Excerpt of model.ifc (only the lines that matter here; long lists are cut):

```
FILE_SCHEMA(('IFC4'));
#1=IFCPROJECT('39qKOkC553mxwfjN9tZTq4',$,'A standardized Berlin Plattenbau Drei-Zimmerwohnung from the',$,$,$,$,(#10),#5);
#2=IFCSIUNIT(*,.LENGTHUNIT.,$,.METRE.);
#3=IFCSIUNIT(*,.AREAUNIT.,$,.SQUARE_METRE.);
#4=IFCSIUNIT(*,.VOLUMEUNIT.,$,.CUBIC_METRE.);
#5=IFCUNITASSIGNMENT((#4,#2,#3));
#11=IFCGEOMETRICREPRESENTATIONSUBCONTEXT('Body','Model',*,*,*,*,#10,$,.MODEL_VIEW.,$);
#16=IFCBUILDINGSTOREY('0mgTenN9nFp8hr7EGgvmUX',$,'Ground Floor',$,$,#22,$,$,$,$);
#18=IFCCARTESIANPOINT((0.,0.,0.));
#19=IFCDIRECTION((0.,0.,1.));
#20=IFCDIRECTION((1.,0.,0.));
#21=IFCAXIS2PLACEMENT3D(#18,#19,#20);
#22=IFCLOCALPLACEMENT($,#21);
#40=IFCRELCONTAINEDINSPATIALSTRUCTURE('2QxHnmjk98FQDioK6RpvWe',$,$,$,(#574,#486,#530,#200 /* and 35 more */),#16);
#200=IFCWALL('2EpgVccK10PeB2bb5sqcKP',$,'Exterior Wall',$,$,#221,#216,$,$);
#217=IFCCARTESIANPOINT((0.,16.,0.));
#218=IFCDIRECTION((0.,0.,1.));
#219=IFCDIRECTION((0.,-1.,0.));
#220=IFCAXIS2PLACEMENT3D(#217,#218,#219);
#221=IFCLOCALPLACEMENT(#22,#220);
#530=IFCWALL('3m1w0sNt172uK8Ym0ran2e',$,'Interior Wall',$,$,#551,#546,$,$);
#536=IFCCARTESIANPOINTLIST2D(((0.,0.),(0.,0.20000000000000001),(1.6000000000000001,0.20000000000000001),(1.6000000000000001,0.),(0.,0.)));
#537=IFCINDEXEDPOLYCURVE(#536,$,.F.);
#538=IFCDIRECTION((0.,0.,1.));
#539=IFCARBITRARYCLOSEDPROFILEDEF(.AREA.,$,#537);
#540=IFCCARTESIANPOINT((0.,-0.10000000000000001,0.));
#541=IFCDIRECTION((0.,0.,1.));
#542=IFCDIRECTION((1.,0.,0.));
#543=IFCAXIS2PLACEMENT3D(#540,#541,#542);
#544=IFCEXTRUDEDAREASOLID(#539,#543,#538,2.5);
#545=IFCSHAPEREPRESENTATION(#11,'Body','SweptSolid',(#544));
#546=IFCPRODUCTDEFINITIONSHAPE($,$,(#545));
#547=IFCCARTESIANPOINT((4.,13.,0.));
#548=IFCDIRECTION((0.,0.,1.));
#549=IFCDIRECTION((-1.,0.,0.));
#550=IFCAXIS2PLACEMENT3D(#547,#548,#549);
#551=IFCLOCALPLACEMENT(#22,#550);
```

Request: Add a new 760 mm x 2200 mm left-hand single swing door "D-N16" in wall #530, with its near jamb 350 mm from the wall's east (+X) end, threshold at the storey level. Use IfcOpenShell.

```python
import numpy as np
import ifcopenshell
import ifcopenshell.api.feature
import ifcopenshell.api.geometry
import ifcopenshell.api.root
import ifcopenshell.api.spatial
import ifcopenshell.geom
import ifcopenshell.util.element
import ifcopenshell.util.placement
import ifcopenshell.util.representation
import ifcopenshell.util.shape
import ifcopenshell.util.unit

model = ifcopenshell.open("model.ifc")
unit_scale = ifcopenshell.util.unit.calculate_unit_scale(model)
settings = ifcopenshell.geom.settings()


def volume(element):
    """Net volume in cubic metres, openings subtracted."""
    shape = ifcopenshell.geom.create_shape(settings, element)
    return ifcopenshell.util.shape.get_volume(shape.geometry)


wall = model.by_guid("3m1w0sNt172uK8Ym0ran2e")
storey = ifcopenshell.util.element.get_container(wall, ifc_class="IfcBuildingStorey")
context = ifcopenshell.util.representation.get_context(model, "Model", "Body", "MODEL_VIEW")
before = volume(wall)

width, height, from_end, sill = 0.76, 2.2, 0.35, 0.0  # metres

# The wall runs along its own X axis, and the end named is its -X end.
wall_shape = ifcopenshell.geom.create_shape(settings, wall)
x, y, z = ifcopenshell.util.shape.get_vertices(wall_shape.geometry).T
start = x.min() + from_end
face, thickness = float(y.min()), float(y.max() - y.min())
wall_matrix = ifcopenshell.util.placement.get_local_placement(wall.ObjectPlacement)
level = ifcopenshell.util.placement.get_local_placement(storey.ObjectPlacement)[2, 3]


def in_wall(x, y):
    """Placement at x, y metres in the wall's axes, at sill height."""
    matrix = wall_matrix.copy()
    matrix[:, 3] = wall_matrix @ np.array([x / unit_scale, y / unit_scale, 0.0, 1.0])
    matrix[2, 3] = level + sill / unit_scale
    return matrix


# Opening: a box that overshoots both wall faces by 50 mm.
opening = ifcopenshell.api.root.create_entity(model, ifc_class="IfcOpeningElement", predefined_type="OPENING")
box = ifcopenshell.api.geometry.add_wall_representation(
    model, context=context, length=width, height=height, thickness=thickness + 0.1
)
ifcopenshell.api.geometry.assign_representation(model, product=opening, representation=box)
ifcopenshell.api.geometry.edit_object_placement(model, product=opening, matrix=in_wall(start, face - 0.05), is_si=False)
ifcopenshell.api.feature.add_feature(model, feature=opening, element=wall)

door = ifcopenshell.api.root.create_entity(model, ifc_class="IfcDoor", name="D-N16", predefined_type="DOOR")
door.OverallWidth, door.OverallHeight = width / unit_scale, height / unit_scale
door.OperationType = "SINGLE_SWING_LEFT"
body = ifcopenshell.api.geometry.add_door_representation(
    model,
    context=context,
    overall_width=door.OverallWidth,
    overall_height=door.OverallHeight,
    operation_type="SINGLE_SWING_LEFT",
    lining_properties={"LiningDepth": thickness / unit_scale, "ThresholdDepth": thickness / unit_scale},
)
ifcopenshell.api.geometry.assign_representation(model, product=door, representation=body)
ifcopenshell.api.spatial.assign_container(model, products=[door], relating_structure=storey)
ifcopenshell.api.feature.add_filling(model, opening=opening, element=door)

# The lining spans the wall, so the door starts at the wall face.
ifcopenshell.api.geometry.edit_object_placement(model, product=door, matrix=in_wall(start, face), is_si=False)

after = volume(wall)

print(f"wall volume {before:.3f} -> {after:.3f} m3")

model.write("model_edited.ifc")
```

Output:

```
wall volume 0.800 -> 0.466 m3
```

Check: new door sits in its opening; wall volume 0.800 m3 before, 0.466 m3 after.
